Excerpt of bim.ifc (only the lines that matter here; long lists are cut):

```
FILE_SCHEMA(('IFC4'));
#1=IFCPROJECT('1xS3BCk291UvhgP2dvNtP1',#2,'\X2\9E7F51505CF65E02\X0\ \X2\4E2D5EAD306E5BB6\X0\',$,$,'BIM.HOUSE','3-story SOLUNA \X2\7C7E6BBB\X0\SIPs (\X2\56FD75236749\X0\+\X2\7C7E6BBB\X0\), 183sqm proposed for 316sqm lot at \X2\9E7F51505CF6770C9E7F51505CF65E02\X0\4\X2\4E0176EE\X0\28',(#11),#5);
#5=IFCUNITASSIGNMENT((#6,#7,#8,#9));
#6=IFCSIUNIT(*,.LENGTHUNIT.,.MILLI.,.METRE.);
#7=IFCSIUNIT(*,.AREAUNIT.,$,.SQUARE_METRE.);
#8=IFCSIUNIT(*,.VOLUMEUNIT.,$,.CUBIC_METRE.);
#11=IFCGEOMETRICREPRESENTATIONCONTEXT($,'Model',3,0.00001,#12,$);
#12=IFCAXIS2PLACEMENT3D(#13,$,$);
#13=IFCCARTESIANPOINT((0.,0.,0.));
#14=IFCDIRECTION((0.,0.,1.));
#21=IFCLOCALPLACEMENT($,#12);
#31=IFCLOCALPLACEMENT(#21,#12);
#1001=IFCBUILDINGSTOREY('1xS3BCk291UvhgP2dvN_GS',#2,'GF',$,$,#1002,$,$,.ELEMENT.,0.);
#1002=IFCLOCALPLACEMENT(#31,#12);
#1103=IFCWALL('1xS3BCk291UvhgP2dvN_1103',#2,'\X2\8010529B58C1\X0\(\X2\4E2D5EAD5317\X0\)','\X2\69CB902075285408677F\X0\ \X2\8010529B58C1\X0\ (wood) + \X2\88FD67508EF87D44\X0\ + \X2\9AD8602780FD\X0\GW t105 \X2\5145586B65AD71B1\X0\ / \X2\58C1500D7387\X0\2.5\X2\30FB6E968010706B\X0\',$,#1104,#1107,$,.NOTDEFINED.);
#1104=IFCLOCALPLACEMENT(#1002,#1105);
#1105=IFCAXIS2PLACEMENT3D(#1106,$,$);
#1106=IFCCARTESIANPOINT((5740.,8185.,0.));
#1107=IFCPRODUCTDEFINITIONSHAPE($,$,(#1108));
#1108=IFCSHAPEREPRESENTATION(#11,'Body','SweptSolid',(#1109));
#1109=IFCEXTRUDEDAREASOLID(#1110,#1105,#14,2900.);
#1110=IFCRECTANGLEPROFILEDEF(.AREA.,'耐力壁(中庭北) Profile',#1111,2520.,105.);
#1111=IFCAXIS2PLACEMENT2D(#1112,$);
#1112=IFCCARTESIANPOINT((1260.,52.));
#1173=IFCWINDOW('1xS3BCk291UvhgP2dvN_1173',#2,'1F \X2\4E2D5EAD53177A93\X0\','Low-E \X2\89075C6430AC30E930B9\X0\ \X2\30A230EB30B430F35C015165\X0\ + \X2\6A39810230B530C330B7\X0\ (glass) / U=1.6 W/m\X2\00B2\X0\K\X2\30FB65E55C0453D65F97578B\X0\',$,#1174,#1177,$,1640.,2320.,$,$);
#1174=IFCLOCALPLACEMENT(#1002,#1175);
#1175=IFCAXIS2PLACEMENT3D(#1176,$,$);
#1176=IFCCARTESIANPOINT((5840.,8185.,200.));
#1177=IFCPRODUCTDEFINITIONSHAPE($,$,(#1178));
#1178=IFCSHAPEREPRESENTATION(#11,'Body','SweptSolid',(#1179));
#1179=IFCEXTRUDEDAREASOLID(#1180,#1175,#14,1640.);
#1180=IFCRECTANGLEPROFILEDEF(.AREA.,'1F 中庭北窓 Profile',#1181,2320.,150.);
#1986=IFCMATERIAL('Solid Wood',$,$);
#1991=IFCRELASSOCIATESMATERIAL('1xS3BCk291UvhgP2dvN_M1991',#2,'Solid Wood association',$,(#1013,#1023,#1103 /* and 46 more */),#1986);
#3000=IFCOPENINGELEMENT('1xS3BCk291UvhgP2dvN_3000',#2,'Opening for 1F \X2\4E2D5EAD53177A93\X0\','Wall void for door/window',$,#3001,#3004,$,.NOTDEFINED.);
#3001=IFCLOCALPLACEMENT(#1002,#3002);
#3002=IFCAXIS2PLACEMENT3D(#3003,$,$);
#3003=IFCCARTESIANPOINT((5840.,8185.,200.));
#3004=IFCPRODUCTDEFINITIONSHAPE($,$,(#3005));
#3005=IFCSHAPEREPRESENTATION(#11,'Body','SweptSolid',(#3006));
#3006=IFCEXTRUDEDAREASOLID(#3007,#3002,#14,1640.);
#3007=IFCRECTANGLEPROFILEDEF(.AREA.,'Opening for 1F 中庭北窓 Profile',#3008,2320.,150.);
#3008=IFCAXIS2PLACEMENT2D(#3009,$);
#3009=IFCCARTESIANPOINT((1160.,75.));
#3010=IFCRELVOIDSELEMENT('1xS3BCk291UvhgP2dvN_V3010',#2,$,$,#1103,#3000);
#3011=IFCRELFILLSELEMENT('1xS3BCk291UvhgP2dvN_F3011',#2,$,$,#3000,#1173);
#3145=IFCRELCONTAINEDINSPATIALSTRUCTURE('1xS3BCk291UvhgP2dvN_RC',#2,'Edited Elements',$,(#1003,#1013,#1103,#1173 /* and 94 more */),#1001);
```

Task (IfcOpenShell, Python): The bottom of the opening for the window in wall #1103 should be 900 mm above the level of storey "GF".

```python
import numpy as np
import ifcopenshell
import ifcopenshell.api.geometry
import ifcopenshell.geom
import ifcopenshell.util.element
import ifcopenshell.util.placement
import ifcopenshell.util.shape
import ifcopenshell.util.unit

model = ifcopenshell.open("bim.ifc")
unit_scale = ifcopenshell.util.unit.calculate_unit_scale(model)

window = model.by_guid("1xS3BCk291UvhgP2dvN_1173")
opening = window.FillsVoids[0].RelatingOpeningElement
storey = ifcopenshell.util.element.get_container(window, ifc_class="IfcBuildingStorey")
level = ifcopenshell.util.placement.get_local_placement(storey.ObjectPlacement)[2, 3]

# The opening's origin need not be at the sill, so measure its lowest point.
shape = ifcopenshell.geom.create_shape(ifcopenshell.geom.settings(), opening)
bottom = ifcopenshell.util.shape.get_shape_bottom_elevation(shape, shape.geometry) / unit_scale
dz = level + 0.9 / unit_scale - bottom

shift = np.array([0.0, 0.0, dz])
# The window is not placed relative to its opening, so move both.
for product in (opening, window):
    matrix = ifcopenshell.util.placement.get_local_placement(product.ObjectPlacement)
    matrix[:3, 3] += shift
    ifcopenshell.api.geometry.edit_object_placement(model, product=product, matrix=matrix, is_si=False)

print(f"moved by {dz * unit_scale:+.3f} m")

model.write("bim_v2.ifc")
```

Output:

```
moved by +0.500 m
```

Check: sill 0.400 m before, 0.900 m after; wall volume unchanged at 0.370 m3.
